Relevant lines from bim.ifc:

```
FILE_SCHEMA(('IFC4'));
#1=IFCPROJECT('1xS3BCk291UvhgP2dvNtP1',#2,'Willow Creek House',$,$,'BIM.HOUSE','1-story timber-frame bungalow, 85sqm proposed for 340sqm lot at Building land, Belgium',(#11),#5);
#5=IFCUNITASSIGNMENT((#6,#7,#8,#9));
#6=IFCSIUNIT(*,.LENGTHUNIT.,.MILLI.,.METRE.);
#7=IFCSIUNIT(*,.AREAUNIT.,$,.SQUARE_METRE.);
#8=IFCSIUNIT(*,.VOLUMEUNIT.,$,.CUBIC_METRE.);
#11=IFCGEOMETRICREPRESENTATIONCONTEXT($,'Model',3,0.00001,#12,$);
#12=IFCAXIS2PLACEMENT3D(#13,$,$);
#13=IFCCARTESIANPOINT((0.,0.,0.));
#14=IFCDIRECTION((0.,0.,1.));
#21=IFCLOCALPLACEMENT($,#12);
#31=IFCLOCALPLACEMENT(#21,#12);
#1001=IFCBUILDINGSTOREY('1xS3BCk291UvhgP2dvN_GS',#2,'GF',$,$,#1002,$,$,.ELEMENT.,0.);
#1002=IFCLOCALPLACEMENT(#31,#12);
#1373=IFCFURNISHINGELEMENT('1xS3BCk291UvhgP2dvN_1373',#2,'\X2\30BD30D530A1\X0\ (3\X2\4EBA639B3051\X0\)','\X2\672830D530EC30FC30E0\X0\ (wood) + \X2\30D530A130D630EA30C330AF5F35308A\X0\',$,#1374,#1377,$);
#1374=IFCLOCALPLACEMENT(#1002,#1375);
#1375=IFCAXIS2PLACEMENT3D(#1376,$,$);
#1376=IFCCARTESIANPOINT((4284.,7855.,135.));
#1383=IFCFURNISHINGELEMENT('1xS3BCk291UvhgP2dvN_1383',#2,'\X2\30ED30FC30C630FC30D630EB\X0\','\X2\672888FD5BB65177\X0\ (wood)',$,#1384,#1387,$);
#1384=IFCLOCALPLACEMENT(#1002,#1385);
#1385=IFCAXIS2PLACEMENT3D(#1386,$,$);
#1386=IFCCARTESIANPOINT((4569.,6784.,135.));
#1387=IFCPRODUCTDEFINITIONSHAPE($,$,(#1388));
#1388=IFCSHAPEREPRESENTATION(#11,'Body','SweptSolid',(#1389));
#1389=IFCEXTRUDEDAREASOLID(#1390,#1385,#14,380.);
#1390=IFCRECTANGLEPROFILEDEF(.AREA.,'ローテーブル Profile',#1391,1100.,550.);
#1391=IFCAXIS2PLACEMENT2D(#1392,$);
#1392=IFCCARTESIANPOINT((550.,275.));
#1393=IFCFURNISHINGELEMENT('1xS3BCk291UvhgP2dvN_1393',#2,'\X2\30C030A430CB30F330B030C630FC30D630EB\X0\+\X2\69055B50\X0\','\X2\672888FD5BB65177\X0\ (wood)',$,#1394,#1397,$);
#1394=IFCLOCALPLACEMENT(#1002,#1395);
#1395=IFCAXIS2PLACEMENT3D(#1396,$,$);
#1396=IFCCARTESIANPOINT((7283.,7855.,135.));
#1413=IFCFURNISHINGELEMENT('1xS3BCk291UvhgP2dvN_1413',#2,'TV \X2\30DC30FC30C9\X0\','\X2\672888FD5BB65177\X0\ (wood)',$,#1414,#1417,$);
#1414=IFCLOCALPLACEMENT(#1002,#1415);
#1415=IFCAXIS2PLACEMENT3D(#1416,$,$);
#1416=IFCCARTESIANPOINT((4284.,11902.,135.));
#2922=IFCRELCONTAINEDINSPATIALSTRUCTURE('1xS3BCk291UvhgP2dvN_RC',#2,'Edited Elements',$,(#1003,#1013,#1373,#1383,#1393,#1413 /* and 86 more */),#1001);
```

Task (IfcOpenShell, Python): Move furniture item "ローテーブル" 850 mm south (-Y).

```python
import ifcopenshell
import ifcopenshell.api.geometry
import ifcopenshell.util.placement
import ifcopenshell.util.unit

model = ifcopenshell.open("bim.ifc")
unit_scale = ifcopenshell.util.unit.calculate_unit_scale(model)

item = model.by_id(1383)
matrix = ifcopenshell.util.placement.get_local_placement(item.ObjectPlacement)
matrix[1, 3] -= 0.85 / unit_scale
ifcopenshell.api.geometry.edit_object_placement(model, product=item, matrix=matrix, is_si=False)

print(ifcopenshell.util.placement.get_local_placement(item.ObjectPlacement).round(3) + 0.0)

model.write("bim_edited.ifc")
```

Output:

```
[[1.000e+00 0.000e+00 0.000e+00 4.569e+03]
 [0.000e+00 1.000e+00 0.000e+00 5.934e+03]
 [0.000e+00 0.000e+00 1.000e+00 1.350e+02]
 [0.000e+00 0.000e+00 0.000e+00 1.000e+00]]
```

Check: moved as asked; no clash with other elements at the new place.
